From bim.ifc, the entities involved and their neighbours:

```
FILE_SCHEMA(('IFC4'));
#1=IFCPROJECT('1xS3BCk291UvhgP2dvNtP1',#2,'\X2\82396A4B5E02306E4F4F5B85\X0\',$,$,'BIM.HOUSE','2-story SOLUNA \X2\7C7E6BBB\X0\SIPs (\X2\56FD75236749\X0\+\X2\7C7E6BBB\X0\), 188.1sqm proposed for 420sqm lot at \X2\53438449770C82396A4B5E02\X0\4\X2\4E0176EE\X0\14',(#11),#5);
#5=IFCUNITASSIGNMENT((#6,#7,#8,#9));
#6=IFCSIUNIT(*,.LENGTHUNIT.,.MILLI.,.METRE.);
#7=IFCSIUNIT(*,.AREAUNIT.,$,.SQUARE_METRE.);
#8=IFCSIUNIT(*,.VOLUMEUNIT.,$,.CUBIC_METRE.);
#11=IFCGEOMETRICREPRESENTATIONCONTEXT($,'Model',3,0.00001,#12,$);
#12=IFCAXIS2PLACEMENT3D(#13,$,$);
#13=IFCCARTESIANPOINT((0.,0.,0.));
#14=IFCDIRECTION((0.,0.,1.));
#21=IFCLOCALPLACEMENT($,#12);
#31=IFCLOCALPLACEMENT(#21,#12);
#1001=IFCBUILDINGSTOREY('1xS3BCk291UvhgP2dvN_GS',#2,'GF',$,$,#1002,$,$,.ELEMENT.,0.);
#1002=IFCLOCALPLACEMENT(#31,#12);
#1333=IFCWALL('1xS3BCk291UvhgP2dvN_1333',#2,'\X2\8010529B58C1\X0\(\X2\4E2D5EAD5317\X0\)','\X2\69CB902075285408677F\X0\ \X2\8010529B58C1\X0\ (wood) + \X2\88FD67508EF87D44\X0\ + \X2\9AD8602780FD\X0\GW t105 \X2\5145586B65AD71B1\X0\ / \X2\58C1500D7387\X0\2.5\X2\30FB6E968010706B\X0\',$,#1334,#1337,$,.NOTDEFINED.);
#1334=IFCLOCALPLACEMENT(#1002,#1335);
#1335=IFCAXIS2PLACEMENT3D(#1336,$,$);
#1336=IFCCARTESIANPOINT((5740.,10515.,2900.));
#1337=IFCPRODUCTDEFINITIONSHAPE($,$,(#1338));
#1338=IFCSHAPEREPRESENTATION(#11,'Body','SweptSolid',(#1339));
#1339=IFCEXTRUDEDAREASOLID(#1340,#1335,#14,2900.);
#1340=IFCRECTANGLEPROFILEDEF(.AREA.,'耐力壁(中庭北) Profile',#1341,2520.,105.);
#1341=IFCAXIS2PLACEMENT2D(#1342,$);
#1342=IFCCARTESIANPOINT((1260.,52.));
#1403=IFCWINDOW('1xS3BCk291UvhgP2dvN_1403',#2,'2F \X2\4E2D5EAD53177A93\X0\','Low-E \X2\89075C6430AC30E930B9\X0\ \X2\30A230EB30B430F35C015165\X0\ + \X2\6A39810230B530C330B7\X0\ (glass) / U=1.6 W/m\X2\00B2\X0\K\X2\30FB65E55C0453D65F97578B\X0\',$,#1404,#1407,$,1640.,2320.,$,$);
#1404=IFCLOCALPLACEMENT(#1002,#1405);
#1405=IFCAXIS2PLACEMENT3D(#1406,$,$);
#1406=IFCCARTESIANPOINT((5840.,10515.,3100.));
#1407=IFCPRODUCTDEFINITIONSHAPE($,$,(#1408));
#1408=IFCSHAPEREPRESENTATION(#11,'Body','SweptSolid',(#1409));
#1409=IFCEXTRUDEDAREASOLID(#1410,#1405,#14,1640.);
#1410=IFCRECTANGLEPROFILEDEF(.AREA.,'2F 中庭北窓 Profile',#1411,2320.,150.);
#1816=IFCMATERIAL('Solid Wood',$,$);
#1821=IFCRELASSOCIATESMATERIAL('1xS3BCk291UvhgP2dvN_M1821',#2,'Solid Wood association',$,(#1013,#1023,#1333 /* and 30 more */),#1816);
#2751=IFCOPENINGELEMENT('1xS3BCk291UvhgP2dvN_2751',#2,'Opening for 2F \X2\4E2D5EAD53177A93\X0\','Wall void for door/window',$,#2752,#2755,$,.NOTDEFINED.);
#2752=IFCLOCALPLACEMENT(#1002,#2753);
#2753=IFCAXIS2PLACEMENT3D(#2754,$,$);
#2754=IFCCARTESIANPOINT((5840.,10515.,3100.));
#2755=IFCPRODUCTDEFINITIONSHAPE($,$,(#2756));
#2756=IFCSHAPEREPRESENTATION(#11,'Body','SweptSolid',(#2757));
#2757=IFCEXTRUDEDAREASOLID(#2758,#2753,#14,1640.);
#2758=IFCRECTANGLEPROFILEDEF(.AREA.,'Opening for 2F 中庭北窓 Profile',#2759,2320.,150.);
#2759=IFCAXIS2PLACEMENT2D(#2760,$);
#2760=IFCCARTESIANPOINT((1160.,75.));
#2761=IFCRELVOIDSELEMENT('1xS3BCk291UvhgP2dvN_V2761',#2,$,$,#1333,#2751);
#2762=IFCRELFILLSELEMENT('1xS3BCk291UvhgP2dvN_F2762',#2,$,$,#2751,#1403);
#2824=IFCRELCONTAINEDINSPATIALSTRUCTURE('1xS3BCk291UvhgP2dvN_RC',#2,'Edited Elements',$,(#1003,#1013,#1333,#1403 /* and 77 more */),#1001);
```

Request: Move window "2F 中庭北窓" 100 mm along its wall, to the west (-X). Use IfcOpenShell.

```python
import ifcopenshell
import ifcopenshell.api.geometry
import ifcopenshell.util.placement
import ifcopenshell.util.unit

model = ifcopenshell.open("bim.ifc")
unit_scale = ifcopenshell.util.unit.calculate_unit_scale(model)

window = model.by_guid("1xS3BCk291UvhgP2dvN_1403")
opening = window.FillsVoids[0].RelatingOpeningElement
wall = opening.VoidsElements[0].RelatingBuildingElement

wall_matrix = ifcopenshell.util.placement.get_local_placement(wall.ObjectPlacement)
shift = wall_matrix[:3, 0] * -0.1 / unit_scale
before = ifcopenshell.util.placement.get_local_placement(window.ObjectPlacement)[:3, 3].copy()

# The window is not placed relative to its opening, so move both.
for product in (opening, window):
    matrix = ifcopenshell.util.placement.get_local_placement(product.ObjectPlacement)
    matrix[:3, 3] += shift
    ifcopenshell.api.geometry.edit_object_placement(model, product=product, matrix=matrix, is_si=False)

after = ifcopenshell.util.placement.get_local_placement(window.ObjectPlacement)[:3, 3]
print("window moved by", (after - before).round(3) + 0.0)

model.write("bim_edited.ifc")
```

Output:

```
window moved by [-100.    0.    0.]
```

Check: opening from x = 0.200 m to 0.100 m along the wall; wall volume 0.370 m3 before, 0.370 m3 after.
